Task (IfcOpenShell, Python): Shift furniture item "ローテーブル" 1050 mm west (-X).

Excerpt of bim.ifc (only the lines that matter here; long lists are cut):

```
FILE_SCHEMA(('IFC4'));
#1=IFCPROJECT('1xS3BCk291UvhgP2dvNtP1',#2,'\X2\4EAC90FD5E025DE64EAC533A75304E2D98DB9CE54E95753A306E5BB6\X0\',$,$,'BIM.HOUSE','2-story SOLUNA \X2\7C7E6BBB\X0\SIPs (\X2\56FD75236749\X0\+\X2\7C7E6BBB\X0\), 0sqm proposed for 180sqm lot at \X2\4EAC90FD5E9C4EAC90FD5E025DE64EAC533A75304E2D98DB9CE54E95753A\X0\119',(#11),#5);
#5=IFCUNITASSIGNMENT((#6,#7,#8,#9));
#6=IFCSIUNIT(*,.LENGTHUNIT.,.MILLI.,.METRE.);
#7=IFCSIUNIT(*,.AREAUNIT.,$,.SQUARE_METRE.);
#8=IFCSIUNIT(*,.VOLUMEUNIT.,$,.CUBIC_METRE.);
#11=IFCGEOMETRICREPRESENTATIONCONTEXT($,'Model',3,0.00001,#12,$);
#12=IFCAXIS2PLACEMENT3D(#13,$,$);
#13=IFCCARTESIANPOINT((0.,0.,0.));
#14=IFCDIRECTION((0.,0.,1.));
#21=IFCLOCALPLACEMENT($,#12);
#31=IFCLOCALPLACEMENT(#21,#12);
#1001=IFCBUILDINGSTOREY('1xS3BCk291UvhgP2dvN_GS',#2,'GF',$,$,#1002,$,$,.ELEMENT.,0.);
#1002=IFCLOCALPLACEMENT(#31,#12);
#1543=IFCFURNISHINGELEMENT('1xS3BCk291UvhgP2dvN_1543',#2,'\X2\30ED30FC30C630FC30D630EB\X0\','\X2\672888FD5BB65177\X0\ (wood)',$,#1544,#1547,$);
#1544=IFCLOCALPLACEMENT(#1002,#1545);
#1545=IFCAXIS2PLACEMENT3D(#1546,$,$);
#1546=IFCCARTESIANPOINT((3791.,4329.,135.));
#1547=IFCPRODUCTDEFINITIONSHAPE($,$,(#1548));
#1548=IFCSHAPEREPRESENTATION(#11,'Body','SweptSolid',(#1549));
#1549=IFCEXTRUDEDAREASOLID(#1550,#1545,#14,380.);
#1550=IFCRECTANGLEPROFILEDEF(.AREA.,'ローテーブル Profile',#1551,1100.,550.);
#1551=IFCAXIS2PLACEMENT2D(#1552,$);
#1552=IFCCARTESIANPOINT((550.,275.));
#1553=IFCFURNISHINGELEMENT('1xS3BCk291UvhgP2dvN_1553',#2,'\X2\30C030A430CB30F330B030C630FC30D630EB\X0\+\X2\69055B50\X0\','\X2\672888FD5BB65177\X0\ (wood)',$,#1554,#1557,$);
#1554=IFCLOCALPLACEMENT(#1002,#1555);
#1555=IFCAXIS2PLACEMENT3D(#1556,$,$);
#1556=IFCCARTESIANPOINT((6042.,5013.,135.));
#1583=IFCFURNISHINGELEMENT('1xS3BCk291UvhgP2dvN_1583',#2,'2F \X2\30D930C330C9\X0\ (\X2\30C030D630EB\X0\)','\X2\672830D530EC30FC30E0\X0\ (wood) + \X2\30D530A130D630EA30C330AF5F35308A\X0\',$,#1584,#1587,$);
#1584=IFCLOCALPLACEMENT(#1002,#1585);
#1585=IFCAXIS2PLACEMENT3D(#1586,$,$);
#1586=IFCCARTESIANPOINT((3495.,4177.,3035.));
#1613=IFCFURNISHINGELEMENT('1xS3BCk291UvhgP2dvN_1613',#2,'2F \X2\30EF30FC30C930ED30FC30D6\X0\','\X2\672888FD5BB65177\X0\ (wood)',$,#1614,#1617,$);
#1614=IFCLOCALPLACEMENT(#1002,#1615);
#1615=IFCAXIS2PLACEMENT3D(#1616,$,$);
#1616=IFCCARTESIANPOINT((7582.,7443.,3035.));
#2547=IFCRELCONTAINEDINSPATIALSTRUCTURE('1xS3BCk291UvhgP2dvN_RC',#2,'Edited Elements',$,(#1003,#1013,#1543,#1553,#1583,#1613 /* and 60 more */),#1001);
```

```python
import ifcopenshell
import ifcopenshell.api.geometry
import ifcopenshell.util.placement

model = ifcopenshell.open("bim.ifc")

item = model.by_guid("1xS3BCk291UvhgP2dvN_1543")
matrix = ifcopenshell.util.placement.get_local_placement(item.ObjectPlacement)
matrix[0, 3] -= 1050.0
ifcopenshell.api.geometry.edit_object_placement(model, product=item, matrix=matrix, is_si=False)

print(ifcopenshell.util.placement.get_local_placement(item.ObjectPlacement).round(3) + 0.0)

model.write("bim_v2.ifc")
```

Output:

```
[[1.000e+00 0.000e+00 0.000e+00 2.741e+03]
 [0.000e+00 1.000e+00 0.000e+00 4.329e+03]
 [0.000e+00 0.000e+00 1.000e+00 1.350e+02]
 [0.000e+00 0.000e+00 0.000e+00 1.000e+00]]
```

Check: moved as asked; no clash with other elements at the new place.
